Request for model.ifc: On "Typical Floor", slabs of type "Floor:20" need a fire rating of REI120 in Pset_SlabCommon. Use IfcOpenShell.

First a look at what the model holds.

```python
import ifcopenshell
import ifcopenshell.util.element

model = ifcopenshell.open("model.ifc")
print(model.schema)
storey = next(s for s in model.by_type("IfcBuildingStorey") if s.Name == "Typical Floor")
slabs = [e for e in ifcopenshell.util.element.get_decomposition(storey) if e.is_a("IfcSlab")]
seen = {}
for e in slabs:
    element_type = ifcopenshell.util.element.get_type(e)
    key = (element_type.Name if element_type != e and element_type else None, ifcopenshell.util.element.get_pset(e, "Pset_SlabCommon", "FireRating"))
    seen[key] = seen.get(key, 0) + 1
for (name, value), count in sorted(seen.items(), key=str):
    print(count, "x", name, "|", value)
```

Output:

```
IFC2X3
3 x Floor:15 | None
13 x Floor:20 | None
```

```python
import ifcopenshell
import ifcopenshell.api.pset
import ifcopenshell.util.element

model = ifcopenshell.open("model.ifc")

storey = next(s for s in model.by_type("IfcBuildingStorey") if s.Name == "Typical Floor")
slabs = [e for e in ifcopenshell.util.element.get_decomposition(storey) if e.is_a("IfcSlab")]

count = 0
for e in slabs:
    element_type = ifcopenshell.util.element.get_type(e)
    if element_type in (None, e) or element_type.Name != "Floor:20":
        continue
    # add_pset returns the element's existing set when there is one.
    pset = ifcopenshell.api.pset.add_pset(model, product=e, name="Pset_SlabCommon")
    ifcopenshell.api.pset.edit_pset(model, pset=pset, properties={"FireRating": "REI120"})
    count += 1

print(count, "slabs updated")

model.write("model_rev.ifc")
```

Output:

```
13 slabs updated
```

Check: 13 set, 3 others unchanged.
